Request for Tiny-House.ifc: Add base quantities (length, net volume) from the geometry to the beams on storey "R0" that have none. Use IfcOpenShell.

First a look at what the model holds.

```python
import ifcopenshell
import ifcopenshell.util.element
import ifcopenshell.util.unit

model = ifcopenshell.open("Tiny-House.ifc")
print(model.schema)
for unit_type in ("LENGTHUNIT", "AREAUNIT", "VOLUMEUNIT"):
    print(unit_type, ifcopenshell.util.unit.calculate_unit_scale(model, unit_type))
storey = next(s for s in model.by_type("IfcBuildingStorey") if s.Name == "R0")
beams = [e for e in ifcopenshell.util.element.get_decomposition(storey) if e.is_a("IfcBeam")]
for e in sorted(beams, key=lambda e: e.id()):
    print(e.id(), e.is_a(), e.Name, list(ifcopenshell.util.element.get_psets(e, qtos_only=True)), sep=" | ")
```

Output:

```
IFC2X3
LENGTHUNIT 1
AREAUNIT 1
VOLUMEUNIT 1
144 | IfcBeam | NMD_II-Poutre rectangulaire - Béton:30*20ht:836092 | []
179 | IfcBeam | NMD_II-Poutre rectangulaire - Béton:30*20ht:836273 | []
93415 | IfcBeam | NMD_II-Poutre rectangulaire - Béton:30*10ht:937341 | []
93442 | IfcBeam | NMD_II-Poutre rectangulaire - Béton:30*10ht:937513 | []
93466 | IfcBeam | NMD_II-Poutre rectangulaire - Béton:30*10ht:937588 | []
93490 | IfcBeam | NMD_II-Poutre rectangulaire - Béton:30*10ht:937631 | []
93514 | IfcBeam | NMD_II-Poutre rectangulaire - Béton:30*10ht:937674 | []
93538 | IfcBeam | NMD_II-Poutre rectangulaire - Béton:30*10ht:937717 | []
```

```python
import ifcopenshell
import ifcopenshell.api.pset
import ifcopenshell.geom
import ifcopenshell.util.element
import ifcopenshell.util.shape
import ifcopenshell.util.unit

model = ifcopenshell.open("Tiny-House.ifc")
unit_scale = ifcopenshell.util.unit.calculate_unit_scale(model)
volume_scale = ifcopenshell.util.unit.calculate_unit_scale(model, "VOLUMEUNIT")
settings = ifcopenshell.geom.settings()

storey = next(s for s in model.by_type("IfcBuildingStorey") if s.Name == "R0")
beams = [e for e in ifcopenshell.util.element.get_decomposition(storey) if e.is_a("IfcBeam")]

for e in sorted(beams, key=lambda e: e.id()):
    if ifcopenshell.util.element.get_psets(e, qtos_only=True, should_inherit=False):
        continue
    # Geometry comes back in metres, in the element's own axes.
    shape = ifcopenshell.geom.create_shape(settings, e)
    values = {
        "Length": ifcopenshell.util.shape.get_max_xyz(shape.geometry) / unit_scale,
        "NetVolume": ifcopenshell.util.shape.get_volume(shape.geometry) / volume_scale,
    }
    qto = ifcopenshell.api.pset.add_qto(model, product=e, name="BaseQuantities")
    ifcopenshell.api.pset.edit_qto(model, qto=qto, properties=values)
    print(e.id(), {k: round(v, 3) for k, v in values.items()})

model.write("Tiny-House_rev.ifc")
```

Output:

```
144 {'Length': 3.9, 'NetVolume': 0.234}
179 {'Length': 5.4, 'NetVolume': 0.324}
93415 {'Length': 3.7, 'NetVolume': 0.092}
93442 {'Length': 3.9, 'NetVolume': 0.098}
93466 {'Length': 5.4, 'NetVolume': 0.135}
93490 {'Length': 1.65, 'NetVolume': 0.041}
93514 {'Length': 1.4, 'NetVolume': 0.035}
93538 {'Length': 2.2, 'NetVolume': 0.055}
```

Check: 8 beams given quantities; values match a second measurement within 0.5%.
